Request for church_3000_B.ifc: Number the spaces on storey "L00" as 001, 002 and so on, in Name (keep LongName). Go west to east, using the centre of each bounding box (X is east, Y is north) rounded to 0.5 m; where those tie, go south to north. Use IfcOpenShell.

First a look at what the model holds.

```python
import ifcopenshell
import ifcopenshell.util.element
import ifcopenshell.util.placement

model = ifcopenshell.open("church_3000_B.ifc")
print(model.schema)
storey = next(s for s in model.by_type("IfcBuildingStorey") if s.Name == "L00")
spaces = [e for e in ifcopenshell.util.element.get_decomposition(storey) if e.is_a("IfcSpace")]
for e in sorted(spaces, key=lambda e: e.id()):
    origin = ifcopenshell.util.placement.get_local_placement(e.ObjectPlacement)[:3, 3]
    print(e.id(), e.Name, e.LongName, origin.round(2) + 0.0, sep=" | ")
```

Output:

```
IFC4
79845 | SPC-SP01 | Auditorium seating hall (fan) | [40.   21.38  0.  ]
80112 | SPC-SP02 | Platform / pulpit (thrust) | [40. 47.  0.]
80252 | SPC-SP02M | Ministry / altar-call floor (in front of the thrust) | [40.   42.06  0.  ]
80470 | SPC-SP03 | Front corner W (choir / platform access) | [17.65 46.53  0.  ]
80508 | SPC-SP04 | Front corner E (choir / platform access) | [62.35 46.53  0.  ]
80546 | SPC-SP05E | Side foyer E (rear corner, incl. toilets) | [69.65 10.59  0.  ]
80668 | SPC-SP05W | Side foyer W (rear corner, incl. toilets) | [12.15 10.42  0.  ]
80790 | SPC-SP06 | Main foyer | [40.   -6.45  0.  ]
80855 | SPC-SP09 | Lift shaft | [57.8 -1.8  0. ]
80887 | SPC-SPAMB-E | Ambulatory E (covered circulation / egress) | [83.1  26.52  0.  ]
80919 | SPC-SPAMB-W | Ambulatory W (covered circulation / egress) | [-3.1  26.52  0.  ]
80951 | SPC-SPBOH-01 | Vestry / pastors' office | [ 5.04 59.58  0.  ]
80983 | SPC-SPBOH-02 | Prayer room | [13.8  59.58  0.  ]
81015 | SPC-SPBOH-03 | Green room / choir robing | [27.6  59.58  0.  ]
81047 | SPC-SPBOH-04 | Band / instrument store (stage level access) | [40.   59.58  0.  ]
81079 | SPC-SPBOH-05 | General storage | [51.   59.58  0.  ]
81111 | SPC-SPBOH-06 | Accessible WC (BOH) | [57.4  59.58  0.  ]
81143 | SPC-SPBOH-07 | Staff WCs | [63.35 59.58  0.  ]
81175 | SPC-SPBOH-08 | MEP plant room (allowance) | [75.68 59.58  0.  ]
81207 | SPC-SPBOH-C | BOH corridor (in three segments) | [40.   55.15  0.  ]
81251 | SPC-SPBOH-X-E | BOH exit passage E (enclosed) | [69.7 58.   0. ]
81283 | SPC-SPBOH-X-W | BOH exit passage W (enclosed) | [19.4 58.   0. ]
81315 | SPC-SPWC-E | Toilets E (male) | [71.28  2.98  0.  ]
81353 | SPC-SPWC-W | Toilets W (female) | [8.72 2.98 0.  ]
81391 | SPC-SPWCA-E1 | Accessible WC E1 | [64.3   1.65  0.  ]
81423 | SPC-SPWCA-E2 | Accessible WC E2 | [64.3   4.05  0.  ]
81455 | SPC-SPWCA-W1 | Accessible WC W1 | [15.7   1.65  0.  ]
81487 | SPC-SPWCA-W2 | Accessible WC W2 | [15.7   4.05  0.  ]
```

```python
import ifcopenshell
import ifcopenshell.geom
import ifcopenshell.util.element
import ifcopenshell.util.shape

model = ifcopenshell.open("church_3000_B.ifc")
settings = ifcopenshell.geom.settings()
settings.set("use-world-coords", True)


def centre(element):
    shape = ifcopenshell.geom.create_shape(settings, element)
    return ifcopenshell.util.shape.get_bbox_centroid(shape.geometry)


storey = next(s for s in model.by_type("IfcBuildingStorey") if s.Name == "L00")
spaces = [e for e in ifcopenshell.util.element.get_decomposition(storey) if e.is_a("IfcSpace")]

# Insertion points can sit at a corner or the storey origin, so sort by the geometry (in metres).
centres = {e: centre(e) for e in spaces}
spaces.sort(key=lambda e: (round(centres[e][0] / 0.5), centres[e][1]))

for i, e in enumerate(spaces, start=1):
    number = f"0{i:02d}"
    e.Name = number
    print(e.id(), number)

model.write("church_3000_B-out.ifc")
```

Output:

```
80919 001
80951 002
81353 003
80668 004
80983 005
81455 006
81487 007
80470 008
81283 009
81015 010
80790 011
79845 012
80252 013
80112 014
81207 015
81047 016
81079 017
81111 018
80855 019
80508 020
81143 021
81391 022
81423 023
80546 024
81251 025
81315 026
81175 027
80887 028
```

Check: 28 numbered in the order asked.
